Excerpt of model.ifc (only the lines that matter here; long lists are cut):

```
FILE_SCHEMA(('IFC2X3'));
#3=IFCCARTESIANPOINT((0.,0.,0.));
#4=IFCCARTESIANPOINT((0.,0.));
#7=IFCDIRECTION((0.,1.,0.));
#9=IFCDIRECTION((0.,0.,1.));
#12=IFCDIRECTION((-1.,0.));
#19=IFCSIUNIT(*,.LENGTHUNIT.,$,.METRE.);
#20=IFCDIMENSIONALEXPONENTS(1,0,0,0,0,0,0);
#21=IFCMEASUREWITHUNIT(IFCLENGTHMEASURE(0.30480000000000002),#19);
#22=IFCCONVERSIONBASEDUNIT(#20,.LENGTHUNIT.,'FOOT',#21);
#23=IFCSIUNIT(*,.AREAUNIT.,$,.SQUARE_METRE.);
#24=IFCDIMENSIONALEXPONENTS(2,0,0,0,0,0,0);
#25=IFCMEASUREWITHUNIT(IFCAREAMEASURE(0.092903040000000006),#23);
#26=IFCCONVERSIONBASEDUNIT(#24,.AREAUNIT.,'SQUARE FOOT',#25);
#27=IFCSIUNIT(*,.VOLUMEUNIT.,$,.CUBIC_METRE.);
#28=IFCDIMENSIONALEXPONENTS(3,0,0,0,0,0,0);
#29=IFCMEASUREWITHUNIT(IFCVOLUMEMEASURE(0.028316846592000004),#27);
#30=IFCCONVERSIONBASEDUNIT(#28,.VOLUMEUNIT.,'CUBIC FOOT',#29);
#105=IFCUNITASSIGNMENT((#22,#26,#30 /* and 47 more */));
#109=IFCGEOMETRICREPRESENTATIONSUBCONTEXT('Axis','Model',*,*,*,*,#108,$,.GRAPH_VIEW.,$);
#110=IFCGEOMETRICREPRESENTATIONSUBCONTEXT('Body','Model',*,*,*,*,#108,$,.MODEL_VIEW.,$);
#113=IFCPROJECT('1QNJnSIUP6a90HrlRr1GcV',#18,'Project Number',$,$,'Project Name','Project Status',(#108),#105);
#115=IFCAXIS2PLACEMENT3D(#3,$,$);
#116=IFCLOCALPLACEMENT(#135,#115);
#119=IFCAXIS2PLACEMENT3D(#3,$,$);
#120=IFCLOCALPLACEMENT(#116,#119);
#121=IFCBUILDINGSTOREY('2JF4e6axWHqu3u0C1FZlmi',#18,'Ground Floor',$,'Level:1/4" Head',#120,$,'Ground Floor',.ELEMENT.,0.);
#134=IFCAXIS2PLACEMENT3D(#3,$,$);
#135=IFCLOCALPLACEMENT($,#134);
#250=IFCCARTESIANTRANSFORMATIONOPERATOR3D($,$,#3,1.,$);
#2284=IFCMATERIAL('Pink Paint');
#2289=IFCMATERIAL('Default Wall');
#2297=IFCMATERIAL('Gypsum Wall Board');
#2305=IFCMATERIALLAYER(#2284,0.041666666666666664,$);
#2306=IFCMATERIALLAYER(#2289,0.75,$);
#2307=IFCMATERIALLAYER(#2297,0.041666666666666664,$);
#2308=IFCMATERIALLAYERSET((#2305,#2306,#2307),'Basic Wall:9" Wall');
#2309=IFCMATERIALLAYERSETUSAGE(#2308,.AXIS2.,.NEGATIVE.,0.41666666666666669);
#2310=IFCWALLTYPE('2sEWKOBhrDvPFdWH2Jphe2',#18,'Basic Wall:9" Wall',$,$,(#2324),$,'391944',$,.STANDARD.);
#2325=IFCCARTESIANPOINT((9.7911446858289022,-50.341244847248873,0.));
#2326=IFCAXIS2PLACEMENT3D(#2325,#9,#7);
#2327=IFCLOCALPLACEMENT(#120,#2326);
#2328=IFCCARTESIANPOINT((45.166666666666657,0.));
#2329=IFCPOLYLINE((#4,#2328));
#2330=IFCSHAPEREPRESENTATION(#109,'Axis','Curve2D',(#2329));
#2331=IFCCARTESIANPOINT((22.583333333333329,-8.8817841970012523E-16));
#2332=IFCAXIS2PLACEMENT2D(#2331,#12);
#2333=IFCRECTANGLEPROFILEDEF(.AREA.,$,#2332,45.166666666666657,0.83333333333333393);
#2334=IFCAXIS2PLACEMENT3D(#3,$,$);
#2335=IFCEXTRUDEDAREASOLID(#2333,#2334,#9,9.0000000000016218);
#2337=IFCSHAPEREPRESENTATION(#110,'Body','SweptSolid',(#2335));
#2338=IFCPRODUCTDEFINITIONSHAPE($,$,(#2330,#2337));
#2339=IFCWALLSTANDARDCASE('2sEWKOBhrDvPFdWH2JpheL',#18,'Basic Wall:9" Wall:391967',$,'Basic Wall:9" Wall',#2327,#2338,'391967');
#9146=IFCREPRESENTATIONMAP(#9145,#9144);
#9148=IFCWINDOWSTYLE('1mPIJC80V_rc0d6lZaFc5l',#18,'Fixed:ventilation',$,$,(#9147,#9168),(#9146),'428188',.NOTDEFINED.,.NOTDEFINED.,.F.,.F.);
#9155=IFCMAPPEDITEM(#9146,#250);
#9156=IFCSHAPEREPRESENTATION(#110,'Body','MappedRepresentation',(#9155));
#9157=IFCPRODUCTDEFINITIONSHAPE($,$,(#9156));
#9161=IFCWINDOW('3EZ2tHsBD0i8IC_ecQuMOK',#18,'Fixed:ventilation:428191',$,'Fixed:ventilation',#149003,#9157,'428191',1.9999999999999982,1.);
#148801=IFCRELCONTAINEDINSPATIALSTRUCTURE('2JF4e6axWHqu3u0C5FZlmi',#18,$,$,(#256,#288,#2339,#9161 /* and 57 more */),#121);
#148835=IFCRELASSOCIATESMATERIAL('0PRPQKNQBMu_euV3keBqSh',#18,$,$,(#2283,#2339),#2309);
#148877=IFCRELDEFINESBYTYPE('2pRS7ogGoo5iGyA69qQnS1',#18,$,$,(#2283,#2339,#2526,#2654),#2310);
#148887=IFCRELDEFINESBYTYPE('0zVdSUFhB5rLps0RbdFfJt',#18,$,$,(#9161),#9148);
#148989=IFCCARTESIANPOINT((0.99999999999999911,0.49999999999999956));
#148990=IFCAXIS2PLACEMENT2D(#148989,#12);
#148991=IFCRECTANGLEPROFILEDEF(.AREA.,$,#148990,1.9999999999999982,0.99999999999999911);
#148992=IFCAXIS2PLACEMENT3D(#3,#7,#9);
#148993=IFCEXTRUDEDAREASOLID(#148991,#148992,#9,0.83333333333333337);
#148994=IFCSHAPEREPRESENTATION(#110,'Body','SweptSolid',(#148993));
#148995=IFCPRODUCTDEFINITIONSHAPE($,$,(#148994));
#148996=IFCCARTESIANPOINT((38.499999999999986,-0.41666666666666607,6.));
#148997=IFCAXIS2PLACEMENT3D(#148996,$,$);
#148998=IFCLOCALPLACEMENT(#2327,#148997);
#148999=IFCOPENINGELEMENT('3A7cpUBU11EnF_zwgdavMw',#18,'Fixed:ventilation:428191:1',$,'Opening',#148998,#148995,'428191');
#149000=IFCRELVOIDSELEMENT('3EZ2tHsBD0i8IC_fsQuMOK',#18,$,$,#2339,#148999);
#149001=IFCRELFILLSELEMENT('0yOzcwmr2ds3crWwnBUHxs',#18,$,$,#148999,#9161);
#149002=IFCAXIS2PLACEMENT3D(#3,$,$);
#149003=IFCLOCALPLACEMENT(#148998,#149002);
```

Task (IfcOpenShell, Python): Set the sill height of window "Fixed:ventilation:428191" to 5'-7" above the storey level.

```python
import numpy as np
import ifcopenshell
import ifcopenshell.api.geometry
import ifcopenshell.geom
import ifcopenshell.util.element
import ifcopenshell.util.placement
import ifcopenshell.util.shape
import ifcopenshell.util.unit

model = ifcopenshell.open("model.ifc")
unit_scale = ifcopenshell.util.unit.calculate_unit_scale(model)

window = model.by_guid("3EZ2tHsBD0i8IC_ecQuMOK")
opening = window.FillsVoids[0].RelatingOpeningElement
storey = ifcopenshell.util.element.get_container(window, ifc_class="IfcBuildingStorey")
level = ifcopenshell.util.placement.get_local_placement(storey.ObjectPlacement)[2, 3]

# The opening's origin need not be at the sill, so measure its lowest point.
shape = ifcopenshell.geom.create_shape(ifcopenshell.geom.settings(), opening)
bottom = ifcopenshell.util.shape.get_shape_bottom_elevation(shape, shape.geometry) / unit_scale
dz = level + 67 * 0.0254 / unit_scale - bottom

shift = np.array([0.0, 0.0, dz])
# The window is placed relative to its opening, so it follows when the opening moves.
matrix = ifcopenshell.util.placement.get_local_placement(opening.ObjectPlacement)
matrix[:3, 3] += shift
ifcopenshell.api.geometry.edit_object_placement(
    model, product=opening, matrix=matrix, is_si=False, should_transform_children=True
)

print(f"moved by {dz * unit_scale:+.3f} m")

model.write("model_updated.ifc")
```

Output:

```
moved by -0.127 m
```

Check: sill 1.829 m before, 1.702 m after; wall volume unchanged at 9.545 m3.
